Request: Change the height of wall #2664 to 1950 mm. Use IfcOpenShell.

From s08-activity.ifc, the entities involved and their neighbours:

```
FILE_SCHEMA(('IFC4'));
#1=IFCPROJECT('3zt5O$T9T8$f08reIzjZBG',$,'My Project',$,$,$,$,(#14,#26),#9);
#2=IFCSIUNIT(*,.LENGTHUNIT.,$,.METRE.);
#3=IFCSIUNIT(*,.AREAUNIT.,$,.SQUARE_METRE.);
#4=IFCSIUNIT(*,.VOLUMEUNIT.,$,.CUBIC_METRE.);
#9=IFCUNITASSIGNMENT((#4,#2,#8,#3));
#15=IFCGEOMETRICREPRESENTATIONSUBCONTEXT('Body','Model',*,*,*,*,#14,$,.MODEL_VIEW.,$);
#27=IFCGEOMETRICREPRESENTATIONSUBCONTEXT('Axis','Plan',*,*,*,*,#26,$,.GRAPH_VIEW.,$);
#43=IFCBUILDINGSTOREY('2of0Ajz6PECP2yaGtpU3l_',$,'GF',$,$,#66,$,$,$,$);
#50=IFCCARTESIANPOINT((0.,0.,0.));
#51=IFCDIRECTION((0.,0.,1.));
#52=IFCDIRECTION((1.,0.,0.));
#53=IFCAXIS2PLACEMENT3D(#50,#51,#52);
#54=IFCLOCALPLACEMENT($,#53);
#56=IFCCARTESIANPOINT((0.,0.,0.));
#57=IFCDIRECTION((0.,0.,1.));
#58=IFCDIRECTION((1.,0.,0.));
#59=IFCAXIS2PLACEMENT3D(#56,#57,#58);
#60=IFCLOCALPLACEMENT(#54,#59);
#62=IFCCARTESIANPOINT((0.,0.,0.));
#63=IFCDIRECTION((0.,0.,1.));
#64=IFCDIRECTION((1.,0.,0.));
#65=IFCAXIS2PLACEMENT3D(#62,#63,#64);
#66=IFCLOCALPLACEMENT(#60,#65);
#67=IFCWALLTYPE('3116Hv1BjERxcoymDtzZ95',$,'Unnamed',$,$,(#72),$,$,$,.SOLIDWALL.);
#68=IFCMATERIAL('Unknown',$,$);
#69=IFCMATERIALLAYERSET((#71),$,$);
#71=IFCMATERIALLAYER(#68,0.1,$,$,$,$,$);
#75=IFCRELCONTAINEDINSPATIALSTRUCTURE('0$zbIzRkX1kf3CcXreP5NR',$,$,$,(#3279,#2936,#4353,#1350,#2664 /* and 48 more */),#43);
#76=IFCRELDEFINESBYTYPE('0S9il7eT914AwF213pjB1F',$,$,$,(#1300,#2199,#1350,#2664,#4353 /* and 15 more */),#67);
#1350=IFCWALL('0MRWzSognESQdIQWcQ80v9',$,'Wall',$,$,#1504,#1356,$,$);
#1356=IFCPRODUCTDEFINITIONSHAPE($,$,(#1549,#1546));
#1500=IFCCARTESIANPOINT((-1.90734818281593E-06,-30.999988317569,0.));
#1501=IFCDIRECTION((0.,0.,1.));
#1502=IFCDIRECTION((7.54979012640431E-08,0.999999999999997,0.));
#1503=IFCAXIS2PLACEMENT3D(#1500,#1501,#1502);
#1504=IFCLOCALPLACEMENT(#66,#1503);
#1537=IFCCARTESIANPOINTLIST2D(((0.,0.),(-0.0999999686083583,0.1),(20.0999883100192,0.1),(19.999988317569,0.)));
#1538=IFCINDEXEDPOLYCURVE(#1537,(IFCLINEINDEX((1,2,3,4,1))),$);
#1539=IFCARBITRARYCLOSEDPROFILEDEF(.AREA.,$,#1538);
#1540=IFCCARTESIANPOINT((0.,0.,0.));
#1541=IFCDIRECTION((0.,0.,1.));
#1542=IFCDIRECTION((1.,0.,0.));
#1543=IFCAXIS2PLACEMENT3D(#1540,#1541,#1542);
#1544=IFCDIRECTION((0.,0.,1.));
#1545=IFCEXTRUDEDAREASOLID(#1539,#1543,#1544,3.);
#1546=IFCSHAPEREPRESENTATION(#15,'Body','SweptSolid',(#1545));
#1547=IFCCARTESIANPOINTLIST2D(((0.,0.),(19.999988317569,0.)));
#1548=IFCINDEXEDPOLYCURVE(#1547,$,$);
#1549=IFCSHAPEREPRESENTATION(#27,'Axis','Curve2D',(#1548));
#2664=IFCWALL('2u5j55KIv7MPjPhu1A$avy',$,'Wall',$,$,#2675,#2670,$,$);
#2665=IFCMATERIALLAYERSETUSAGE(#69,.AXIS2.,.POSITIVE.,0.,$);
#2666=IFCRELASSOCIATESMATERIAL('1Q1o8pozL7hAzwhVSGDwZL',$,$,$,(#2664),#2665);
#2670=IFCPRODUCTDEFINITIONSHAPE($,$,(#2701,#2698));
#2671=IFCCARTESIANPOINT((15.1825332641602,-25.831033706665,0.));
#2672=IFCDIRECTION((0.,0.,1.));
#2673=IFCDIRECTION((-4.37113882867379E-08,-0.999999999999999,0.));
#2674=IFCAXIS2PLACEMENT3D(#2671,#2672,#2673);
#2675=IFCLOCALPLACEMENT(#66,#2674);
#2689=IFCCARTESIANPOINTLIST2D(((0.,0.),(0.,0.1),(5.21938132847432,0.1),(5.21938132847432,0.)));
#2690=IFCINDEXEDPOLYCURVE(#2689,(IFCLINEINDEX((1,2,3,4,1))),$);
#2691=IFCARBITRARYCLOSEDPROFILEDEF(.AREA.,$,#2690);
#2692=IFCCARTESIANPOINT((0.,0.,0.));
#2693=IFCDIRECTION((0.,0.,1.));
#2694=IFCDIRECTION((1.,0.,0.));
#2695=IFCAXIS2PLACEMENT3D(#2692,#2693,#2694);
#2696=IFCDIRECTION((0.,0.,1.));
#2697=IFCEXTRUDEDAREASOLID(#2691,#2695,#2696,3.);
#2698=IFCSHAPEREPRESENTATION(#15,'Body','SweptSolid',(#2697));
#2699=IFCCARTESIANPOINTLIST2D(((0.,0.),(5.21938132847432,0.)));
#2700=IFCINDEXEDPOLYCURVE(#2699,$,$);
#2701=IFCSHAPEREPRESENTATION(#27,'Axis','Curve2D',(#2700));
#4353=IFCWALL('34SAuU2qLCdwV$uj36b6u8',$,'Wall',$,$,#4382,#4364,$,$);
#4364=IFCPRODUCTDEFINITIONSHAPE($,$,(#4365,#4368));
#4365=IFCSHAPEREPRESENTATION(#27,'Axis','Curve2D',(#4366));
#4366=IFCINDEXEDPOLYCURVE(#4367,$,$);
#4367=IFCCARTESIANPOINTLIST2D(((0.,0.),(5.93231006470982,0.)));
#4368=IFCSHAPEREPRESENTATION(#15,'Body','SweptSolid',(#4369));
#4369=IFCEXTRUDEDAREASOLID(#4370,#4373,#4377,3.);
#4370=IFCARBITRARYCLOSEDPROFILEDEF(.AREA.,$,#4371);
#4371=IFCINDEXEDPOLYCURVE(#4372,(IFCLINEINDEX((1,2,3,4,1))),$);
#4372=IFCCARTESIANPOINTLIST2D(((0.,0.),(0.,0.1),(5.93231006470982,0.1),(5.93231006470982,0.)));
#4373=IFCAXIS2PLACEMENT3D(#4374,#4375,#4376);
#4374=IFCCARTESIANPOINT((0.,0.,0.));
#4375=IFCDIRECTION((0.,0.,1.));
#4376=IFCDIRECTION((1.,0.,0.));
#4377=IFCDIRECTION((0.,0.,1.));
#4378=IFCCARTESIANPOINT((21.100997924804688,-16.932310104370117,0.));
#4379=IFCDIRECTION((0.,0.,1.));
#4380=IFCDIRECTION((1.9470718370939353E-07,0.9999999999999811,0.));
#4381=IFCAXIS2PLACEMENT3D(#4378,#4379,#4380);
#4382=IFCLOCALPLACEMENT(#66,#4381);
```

```python
import ifcopenshell
import ifcopenshell.geom
import ifcopenshell.util.representation
import ifcopenshell.util.shape

model = ifcopenshell.open("s08-activity.ifc")
settings = ifcopenshell.geom.settings()


def volume(element):
    """Net volume in cubic metres, openings subtracted."""
    shape = ifcopenshell.geom.create_shape(settings, element)
    return ifcopenshell.util.shape.get_volume(shape.geometry)


wall = model.by_guid("2u5j55KIv7MPjPhu1A$avy")
before = volume(wall)

body = ifcopenshell.util.representation.get_representation(wall, "Model", "Body")
solid = body.Items[0]
old_height = solid.Depth
solid.Depth = 1.95
after = volume(wall)

print(f"height {old_height:g} -> {solid.Depth:g}, volume {before:.3f} -> {after:.3f} m3")

model.write("s08-activity_updated.ifc")
```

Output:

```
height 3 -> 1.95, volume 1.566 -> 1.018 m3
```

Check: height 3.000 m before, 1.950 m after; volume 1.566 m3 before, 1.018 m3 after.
